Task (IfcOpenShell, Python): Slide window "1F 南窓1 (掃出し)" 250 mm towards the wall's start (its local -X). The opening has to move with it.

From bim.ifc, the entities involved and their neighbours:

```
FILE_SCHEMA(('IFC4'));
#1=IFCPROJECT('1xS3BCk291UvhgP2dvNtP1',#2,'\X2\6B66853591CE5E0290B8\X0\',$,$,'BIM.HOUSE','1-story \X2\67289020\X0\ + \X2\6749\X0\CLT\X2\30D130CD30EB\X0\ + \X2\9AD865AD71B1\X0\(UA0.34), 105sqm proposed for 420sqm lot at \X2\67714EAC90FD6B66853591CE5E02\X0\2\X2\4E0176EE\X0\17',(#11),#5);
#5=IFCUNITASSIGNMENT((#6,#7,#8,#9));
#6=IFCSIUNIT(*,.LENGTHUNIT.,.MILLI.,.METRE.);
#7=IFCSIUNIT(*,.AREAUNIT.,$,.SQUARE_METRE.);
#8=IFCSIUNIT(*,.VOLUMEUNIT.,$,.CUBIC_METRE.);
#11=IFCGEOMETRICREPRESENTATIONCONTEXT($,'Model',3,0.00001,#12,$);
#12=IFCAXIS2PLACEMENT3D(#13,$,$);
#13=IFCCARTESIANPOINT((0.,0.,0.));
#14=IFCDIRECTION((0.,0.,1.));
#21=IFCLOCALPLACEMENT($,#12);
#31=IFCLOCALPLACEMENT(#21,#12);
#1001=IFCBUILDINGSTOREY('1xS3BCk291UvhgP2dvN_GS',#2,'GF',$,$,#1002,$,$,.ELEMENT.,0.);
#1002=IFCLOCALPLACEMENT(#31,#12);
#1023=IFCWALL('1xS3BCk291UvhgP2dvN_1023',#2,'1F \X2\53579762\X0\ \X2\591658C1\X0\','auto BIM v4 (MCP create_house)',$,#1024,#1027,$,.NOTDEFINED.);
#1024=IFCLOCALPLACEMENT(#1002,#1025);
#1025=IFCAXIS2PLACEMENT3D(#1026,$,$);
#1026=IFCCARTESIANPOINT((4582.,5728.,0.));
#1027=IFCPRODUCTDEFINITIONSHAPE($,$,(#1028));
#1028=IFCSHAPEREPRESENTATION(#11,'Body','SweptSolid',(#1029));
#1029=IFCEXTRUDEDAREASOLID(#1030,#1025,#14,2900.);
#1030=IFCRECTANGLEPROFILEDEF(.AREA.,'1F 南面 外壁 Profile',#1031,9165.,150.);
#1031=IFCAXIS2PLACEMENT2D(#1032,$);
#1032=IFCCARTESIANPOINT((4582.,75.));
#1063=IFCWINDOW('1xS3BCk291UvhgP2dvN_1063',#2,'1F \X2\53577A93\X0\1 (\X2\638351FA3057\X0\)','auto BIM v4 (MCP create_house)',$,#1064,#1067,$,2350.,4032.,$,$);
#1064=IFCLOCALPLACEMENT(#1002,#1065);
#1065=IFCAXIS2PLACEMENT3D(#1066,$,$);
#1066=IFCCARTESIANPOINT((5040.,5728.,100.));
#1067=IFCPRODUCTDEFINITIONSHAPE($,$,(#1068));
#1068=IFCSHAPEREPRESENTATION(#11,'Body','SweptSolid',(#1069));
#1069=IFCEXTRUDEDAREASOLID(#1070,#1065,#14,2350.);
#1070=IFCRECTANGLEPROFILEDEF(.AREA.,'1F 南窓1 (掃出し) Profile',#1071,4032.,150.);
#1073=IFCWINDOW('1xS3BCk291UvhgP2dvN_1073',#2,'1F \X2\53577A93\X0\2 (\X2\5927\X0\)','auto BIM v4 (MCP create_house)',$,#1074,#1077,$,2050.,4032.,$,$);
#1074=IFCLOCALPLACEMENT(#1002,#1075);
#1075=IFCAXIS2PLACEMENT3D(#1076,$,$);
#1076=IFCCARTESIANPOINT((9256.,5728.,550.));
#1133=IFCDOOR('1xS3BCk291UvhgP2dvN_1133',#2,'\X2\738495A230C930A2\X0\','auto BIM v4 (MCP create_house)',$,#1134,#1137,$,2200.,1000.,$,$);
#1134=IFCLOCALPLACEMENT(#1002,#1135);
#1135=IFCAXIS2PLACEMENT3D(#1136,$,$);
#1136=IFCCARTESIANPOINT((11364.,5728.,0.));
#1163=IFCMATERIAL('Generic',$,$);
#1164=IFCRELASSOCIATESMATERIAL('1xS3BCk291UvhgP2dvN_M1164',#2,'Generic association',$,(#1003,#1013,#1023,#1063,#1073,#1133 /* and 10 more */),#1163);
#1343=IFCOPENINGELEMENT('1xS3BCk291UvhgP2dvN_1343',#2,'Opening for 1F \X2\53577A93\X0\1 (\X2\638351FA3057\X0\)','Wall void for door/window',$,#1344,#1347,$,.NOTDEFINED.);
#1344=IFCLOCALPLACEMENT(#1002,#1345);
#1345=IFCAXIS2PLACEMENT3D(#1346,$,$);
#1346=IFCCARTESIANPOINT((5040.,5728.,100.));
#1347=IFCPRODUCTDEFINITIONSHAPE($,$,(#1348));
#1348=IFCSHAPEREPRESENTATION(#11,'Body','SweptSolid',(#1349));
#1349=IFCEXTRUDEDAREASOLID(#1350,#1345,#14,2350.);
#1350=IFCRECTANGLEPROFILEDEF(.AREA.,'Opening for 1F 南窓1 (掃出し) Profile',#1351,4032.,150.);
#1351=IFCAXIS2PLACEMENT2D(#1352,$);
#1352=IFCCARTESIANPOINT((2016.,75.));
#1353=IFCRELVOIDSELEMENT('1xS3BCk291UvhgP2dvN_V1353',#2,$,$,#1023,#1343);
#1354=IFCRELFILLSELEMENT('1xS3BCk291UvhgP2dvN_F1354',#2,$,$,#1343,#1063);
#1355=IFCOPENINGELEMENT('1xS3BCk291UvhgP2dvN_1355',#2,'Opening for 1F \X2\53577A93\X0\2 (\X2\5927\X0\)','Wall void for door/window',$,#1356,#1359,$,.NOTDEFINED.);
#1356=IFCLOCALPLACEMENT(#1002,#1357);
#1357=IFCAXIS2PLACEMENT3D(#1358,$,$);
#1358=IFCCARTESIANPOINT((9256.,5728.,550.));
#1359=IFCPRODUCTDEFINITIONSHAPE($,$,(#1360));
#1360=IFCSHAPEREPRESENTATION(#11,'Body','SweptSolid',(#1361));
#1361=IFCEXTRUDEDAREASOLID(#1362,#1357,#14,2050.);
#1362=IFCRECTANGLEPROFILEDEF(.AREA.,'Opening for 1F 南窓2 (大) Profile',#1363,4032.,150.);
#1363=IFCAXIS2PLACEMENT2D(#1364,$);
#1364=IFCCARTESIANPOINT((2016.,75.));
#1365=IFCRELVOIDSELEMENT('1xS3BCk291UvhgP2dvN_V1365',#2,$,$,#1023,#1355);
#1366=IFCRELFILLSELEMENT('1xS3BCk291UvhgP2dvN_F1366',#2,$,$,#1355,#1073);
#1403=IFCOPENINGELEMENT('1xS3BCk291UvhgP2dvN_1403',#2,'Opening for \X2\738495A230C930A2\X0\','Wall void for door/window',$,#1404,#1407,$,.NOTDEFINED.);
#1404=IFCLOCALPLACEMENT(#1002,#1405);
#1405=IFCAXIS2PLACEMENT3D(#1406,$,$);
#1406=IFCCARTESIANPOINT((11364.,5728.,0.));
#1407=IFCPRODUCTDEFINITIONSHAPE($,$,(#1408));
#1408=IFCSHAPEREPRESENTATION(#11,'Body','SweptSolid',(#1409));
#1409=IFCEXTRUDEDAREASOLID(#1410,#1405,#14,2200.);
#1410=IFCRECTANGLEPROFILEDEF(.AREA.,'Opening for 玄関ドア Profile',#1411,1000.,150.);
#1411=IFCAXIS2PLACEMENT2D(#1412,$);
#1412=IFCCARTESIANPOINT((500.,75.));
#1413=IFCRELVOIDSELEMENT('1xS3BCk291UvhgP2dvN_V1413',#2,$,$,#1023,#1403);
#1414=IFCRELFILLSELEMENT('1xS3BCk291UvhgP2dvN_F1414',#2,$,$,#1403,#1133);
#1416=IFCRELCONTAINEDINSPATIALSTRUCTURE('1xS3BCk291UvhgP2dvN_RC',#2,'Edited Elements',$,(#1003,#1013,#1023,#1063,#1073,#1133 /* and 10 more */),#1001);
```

```python
import ifcopenshell
import ifcopenshell.api.geometry
import ifcopenshell.util.placement
import ifcopenshell.util.unit

model = ifcopenshell.open("bim.ifc")
unit_scale = ifcopenshell.util.unit.calculate_unit_scale(model)

window = model.by_guid("1xS3BCk291UvhgP2dvN_1063")
opening = window.FillsVoids[0].RelatingOpeningElement
wall = opening.VoidsElements[0].RelatingBuildingElement

wall_matrix = ifcopenshell.util.placement.get_local_placement(wall.ObjectPlacement)
shift = wall_matrix[:3, 0] * -0.25 / unit_scale
before = ifcopenshell.util.placement.get_local_placement(window.ObjectPlacement)[:3, 3].copy()

# The window is not placed relative to its opening, so move both.
for product in (opening, window):
    matrix = ifcopenshell.util.placement.get_local_placement(product.ObjectPlacement)
    matrix[:3, 3] += shift
    ifcopenshell.api.geometry.edit_object_placement(model, product=product, matrix=matrix, is_si=False)

after = ifcopenshell.util.placement.get_local_placement(window.ObjectPlacement)[:3, 3]
print("window moved by", (after - before).round(3) + 0.0)

model.write("bim_updated.ifc")
```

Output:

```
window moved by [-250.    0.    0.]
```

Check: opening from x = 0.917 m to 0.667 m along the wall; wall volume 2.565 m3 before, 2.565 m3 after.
